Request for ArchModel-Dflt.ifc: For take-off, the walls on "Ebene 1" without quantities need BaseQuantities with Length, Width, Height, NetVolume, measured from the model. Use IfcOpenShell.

First a look at what the model holds.

```python
import ifcopenshell
import ifcopenshell.util.element
import ifcopenshell.util.unit

model = ifcopenshell.open("ArchModel-Dflt.ifc")
print(model.schema)
for unit_type in ("LENGTHUNIT", "AREAUNIT", "VOLUMEUNIT"):
    print(unit_type, ifcopenshell.util.unit.calculate_unit_scale(model, unit_type))
storey = next(s for s in model.by_type("IfcBuildingStorey") if s.Name == "Ebene 1")
walls = [e for e in ifcopenshell.util.element.get_decomposition(storey) if e.is_a("IfcWall")]
for e in sorted(walls, key=lambda e: e.id()):
    print(e.id(), e.is_a(), e.Name, list(ifcopenshell.util.element.get_psets(e, qtos_only=True)), sep=" | ")
```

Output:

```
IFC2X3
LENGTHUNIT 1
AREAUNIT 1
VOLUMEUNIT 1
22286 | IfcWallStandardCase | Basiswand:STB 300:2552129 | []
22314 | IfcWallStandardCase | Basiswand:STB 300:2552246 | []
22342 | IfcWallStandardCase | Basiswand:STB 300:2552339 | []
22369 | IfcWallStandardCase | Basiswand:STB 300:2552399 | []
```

```python
import ifcopenshell
import ifcopenshell.api.pset
import ifcopenshell.geom
import ifcopenshell.util.element
import ifcopenshell.util.shape
import ifcopenshell.util.unit

model = ifcopenshell.open("ArchModel-Dflt.ifc")
unit_scale = ifcopenshell.util.unit.calculate_unit_scale(model)
volume_scale = ifcopenshell.util.unit.calculate_unit_scale(model, "VOLUMEUNIT")
settings = ifcopenshell.geom.settings()

storey = next(s for s in model.by_type("IfcBuildingStorey") if s.Name == "Ebene 1")
walls = [e for e in ifcopenshell.util.element.get_decomposition(storey) if e.is_a("IfcWall")]

for e in sorted(walls, key=lambda e: e.id()):
    if ifcopenshell.util.element.get_psets(e, qtos_only=True, should_inherit=False):
        continue
    # Geometry comes back in metres, in the element's own axes.
    shape = ifcopenshell.geom.create_shape(settings, e)
    values = {
        "Length": ifcopenshell.util.shape.get_x(shape.geometry) / unit_scale,
        "Width": ifcopenshell.util.shape.get_y(shape.geometry) / unit_scale,
        "Height": ifcopenshell.util.shape.get_z(shape.geometry) / unit_scale,
        "NetVolume": ifcopenshell.util.shape.get_volume(shape.geometry) / volume_scale,
    }
    qto = ifcopenshell.api.pset.add_qto(model, product=e, name="BaseQuantities")
    ifcopenshell.api.pset.edit_qto(model, qto=qto, properties=values)
    print(e.id(), {k: round(v, 3) for k, v in values.items()})

model.write("ArchModel-Dflt-out.ifc")
```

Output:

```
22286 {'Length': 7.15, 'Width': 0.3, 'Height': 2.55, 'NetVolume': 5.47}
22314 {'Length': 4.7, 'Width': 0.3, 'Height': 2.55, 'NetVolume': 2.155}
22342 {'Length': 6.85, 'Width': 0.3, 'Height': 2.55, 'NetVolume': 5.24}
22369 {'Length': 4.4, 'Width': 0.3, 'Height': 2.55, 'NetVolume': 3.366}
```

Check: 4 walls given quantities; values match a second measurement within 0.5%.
